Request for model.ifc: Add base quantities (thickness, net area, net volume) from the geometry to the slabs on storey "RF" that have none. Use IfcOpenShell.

First a look at what the model holds.

```python
import ifcopenshell
import ifcopenshell.util.element
import ifcopenshell.util.unit

model = ifcopenshell.open("model.ifc")
print(model.schema)
for unit_type in ("LENGTHUNIT", "AREAUNIT", "VOLUMEUNIT"):
    print(unit_type, ifcopenshell.util.unit.calculate_unit_scale(model, unit_type))
storey = next(s for s in model.by_type("IfcBuildingStorey") if s.Name == "RF")
slabs = [e for e in ifcopenshell.util.element.get_decomposition(storey) if e.is_a("IfcSlab")]
for e in sorted(slabs, key=lambda e: e.id()):
    print(e.id(), e.is_a(), e.Name, list(ifcopenshell.util.element.get_psets(e, qtos_only=True)), sep=" | ")
```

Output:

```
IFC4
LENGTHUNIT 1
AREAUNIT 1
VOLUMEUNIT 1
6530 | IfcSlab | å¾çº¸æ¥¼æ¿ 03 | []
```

```python
import ifcopenshell
import ifcopenshell.api.pset
import ifcopenshell.geom
import ifcopenshell.util.element
import ifcopenshell.util.shape
import ifcopenshell.util.unit

model = ifcopenshell.open("model.ifc")
unit_scale = ifcopenshell.util.unit.calculate_unit_scale(model)
area_scale = ifcopenshell.util.unit.calculate_unit_scale(model, "AREAUNIT")
volume_scale = ifcopenshell.util.unit.calculate_unit_scale(model, "VOLUMEUNIT")
settings = ifcopenshell.geom.settings()

storey = next(s for s in model.by_type("IfcBuildingStorey") if s.Name == "RF")
slabs = [e for e in ifcopenshell.util.element.get_decomposition(storey) if e.is_a("IfcSlab")]

for e in sorted(slabs, key=lambda e: e.id()):
    if ifcopenshell.util.element.get_psets(e, qtos_only=True, should_inherit=False):
        continue
    # Geometry comes back in metres, in the element's own axes.
    shape = ifcopenshell.geom.create_shape(settings, e)
    values = {
        "Width": ifcopenshell.util.shape.get_z(shape.geometry) / unit_scale,
        "NetArea": ifcopenshell.util.shape.get_footprint_area(shape.geometry) / area_scale,
        "NetVolume": ifcopenshell.util.shape.get_volume(shape.geometry) / volume_scale,
    }
    qto = ifcopenshell.api.pset.add_qto(model, product=e, name="Qto_SlabBaseQuantities")
    ifcopenshell.api.pset.edit_qto(model, qto=qto, properties=values)
    print(e.id(), {k: round(v, 3) for k, v in values.items()})

model.write("model_rev.ifc")
```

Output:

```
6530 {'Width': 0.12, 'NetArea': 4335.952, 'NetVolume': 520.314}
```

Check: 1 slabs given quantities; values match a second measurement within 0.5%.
